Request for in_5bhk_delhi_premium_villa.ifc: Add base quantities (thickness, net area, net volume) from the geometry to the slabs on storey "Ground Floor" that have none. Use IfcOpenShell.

First a look at what the model holds.

```python
import ifcopenshell
import ifcopenshell.util.element
import ifcopenshell.util.unit

model = ifcopenshell.open("in_5bhk_delhi_premium_villa.ifc")
print(model.schema)
for unit_type in ("LENGTHUNIT", "AREAUNIT", "VOLUMEUNIT"):
    print(unit_type, ifcopenshell.util.unit.calculate_unit_scale(model, unit_type))
storey = next(s for s in model.by_type("IfcBuildingStorey") if s.Name == "Ground Floor")
slabs = [e for e in ifcopenshell.util.element.get_decomposition(storey) if e.is_a("IfcSlab")]
for e in sorted(slabs, key=lambda e: e.id()):
    print(e.id(), e.is_a(), e.Name, list(ifcopenshell.util.element.get_psets(e, qtos_only=True)), sep=" | ")
```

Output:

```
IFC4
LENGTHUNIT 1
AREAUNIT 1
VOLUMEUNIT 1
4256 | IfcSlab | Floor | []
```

```python
import ifcopenshell
import ifcopenshell.api.pset
import ifcopenshell.geom
import ifcopenshell.util.element
import ifcopenshell.util.shape
import ifcopenshell.util.unit

model = ifcopenshell.open("in_5bhk_delhi_premium_villa.ifc")
unit_scale = ifcopenshell.util.unit.calculate_unit_scale(model)
area_scale = ifcopenshell.util.unit.calculate_unit_scale(model, "AREAUNIT")
volume_scale = ifcopenshell.util.unit.calculate_unit_scale(model, "VOLUMEUNIT")
settings = ifcopenshell.geom.settings()

storey = next(s for s in model.by_type("IfcBuildingStorey") if s.Name == "Ground Floor")
slabs = [e for e in ifcopenshell.util.element.get_decomposition(storey) if e.is_a("IfcSlab")]

for e in sorted(slabs, key=lambda e: e.id()):
    if ifcopenshell.util.element.get_psets(e, qtos_only=True, should_inherit=False):
        continue
    # Geometry comes back in metres, in the element's own axes.
    shape = ifcopenshell.geom.create_shape(settings, e)
    values = {
        "Width": ifcopenshell.util.shape.get_z(shape.geometry) / unit_scale,
        "NetArea": ifcopenshell.util.shape.get_footprint_area(shape.geometry) / area_scale,
        "NetVolume": ifcopenshell.util.shape.get_volume(shape.geometry) / volume_scale,
    }
    qto = ifcopenshell.api.pset.add_qto(model, product=e, name="Qto_SlabBaseQuantities")
    ifcopenshell.api.pset.edit_qto(model, qto=qto, properties=values)
    print(e.id(), {k: round(v, 3) for k, v in values.items()})

model.write("in_5bhk_delhi_premium_villa-out.ifc")
```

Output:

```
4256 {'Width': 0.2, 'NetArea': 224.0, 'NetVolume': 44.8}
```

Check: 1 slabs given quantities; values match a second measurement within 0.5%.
